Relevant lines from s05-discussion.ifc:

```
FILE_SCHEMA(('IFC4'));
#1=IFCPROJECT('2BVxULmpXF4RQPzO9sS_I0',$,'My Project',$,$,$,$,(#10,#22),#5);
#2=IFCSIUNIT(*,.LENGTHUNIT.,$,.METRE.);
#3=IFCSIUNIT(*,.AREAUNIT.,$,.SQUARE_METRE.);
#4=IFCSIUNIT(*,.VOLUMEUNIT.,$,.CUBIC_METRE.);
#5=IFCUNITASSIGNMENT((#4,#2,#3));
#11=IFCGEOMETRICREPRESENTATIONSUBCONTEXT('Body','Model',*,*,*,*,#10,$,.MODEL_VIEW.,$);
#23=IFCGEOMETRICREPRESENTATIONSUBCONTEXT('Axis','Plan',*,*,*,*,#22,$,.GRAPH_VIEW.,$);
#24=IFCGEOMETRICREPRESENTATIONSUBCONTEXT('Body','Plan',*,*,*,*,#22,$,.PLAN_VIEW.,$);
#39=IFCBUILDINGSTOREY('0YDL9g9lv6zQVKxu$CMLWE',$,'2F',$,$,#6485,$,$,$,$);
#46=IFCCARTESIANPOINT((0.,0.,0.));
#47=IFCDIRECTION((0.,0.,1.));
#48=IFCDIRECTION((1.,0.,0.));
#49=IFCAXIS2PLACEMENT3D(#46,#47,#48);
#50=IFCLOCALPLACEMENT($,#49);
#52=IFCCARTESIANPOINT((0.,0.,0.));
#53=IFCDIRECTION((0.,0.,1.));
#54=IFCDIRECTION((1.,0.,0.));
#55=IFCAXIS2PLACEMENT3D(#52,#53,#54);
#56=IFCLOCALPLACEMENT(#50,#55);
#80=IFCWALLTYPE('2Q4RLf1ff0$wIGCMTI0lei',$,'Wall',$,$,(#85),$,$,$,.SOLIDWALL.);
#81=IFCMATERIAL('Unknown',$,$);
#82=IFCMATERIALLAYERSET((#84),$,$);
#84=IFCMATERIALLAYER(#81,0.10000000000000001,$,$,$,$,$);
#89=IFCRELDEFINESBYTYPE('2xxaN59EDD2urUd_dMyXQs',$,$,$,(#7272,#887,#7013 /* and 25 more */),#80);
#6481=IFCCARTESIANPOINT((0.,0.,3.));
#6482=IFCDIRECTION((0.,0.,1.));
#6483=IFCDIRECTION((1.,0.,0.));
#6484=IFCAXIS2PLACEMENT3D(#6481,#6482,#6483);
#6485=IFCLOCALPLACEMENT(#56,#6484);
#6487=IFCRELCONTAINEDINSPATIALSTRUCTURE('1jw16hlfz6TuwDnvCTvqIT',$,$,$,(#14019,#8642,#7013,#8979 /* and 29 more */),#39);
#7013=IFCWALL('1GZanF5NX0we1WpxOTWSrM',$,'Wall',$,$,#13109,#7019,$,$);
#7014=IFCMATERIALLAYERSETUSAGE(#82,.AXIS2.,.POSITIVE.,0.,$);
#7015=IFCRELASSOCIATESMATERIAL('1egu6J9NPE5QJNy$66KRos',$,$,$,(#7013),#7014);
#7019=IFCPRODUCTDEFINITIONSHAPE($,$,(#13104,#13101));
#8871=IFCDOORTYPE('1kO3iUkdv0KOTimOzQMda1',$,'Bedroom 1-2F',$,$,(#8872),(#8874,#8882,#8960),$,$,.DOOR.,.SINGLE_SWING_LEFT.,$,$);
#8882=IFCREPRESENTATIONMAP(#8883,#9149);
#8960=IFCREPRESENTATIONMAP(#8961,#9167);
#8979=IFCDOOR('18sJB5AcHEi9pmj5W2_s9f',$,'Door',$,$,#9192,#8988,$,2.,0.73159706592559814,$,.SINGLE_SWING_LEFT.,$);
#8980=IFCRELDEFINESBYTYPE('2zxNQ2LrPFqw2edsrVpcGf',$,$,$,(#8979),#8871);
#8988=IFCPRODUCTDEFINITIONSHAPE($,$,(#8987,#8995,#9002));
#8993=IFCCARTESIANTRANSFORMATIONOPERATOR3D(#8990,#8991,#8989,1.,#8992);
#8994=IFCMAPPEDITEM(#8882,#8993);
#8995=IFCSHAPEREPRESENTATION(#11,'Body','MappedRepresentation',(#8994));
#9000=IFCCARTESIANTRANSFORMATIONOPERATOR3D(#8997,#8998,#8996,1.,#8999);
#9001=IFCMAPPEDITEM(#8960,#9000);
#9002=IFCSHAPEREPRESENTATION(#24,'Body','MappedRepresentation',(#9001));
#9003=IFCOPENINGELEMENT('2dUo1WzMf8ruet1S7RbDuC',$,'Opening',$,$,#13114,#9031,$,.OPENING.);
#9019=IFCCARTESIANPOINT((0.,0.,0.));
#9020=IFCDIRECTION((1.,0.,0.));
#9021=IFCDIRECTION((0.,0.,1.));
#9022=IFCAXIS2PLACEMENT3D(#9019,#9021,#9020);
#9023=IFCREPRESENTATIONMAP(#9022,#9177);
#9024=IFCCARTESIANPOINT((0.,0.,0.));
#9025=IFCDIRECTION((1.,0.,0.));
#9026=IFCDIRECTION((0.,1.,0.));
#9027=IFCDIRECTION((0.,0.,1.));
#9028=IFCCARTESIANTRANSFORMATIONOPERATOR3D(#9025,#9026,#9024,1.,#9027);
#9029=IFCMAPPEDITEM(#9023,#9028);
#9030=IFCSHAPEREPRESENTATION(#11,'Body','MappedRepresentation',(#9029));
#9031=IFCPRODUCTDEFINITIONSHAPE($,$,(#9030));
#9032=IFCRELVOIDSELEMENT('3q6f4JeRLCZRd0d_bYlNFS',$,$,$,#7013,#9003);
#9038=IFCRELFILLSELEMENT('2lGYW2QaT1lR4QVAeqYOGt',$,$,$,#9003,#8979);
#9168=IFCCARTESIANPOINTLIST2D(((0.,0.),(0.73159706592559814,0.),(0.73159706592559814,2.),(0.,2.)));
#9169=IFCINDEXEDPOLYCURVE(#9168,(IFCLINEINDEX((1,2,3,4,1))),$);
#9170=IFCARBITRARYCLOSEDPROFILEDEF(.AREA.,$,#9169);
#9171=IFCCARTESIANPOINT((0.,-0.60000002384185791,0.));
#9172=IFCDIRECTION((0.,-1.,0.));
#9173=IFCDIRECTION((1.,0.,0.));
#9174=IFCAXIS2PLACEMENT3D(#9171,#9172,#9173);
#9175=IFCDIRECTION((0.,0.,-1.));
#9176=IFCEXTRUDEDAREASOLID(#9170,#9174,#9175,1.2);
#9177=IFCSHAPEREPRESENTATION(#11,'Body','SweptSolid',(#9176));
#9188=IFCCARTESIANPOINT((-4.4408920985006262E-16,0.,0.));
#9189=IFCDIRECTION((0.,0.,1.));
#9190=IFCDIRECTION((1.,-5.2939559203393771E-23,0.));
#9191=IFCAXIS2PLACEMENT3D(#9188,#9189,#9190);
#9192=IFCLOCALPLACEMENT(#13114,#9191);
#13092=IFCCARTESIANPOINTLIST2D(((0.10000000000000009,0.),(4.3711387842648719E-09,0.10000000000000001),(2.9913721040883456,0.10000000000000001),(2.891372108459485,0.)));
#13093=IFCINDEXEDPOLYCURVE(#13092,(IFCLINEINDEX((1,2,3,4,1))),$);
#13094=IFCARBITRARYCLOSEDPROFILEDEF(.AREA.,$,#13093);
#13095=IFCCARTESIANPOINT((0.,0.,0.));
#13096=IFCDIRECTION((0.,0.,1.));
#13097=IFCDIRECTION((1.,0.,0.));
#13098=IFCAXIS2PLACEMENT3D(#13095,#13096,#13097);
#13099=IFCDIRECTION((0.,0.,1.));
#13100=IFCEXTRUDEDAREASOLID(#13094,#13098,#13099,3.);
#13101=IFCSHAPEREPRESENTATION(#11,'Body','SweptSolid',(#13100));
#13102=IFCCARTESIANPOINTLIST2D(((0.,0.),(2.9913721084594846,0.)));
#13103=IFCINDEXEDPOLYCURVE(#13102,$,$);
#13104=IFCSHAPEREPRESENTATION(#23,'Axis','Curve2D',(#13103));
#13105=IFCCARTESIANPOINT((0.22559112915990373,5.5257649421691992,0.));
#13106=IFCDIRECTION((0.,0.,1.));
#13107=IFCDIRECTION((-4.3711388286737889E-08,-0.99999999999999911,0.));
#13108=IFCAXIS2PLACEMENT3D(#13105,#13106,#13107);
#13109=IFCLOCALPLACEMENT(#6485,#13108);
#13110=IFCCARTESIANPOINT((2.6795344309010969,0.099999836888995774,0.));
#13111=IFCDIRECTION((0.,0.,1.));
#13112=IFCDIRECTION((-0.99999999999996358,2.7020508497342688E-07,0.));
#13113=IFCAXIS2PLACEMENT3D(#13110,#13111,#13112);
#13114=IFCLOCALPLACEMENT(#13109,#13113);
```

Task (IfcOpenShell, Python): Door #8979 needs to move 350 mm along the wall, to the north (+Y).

```python
import ifcopenshell
import ifcopenshell.api.geometry
import ifcopenshell.util.placement
import ifcopenshell.util.unit

model = ifcopenshell.open("s05-discussion.ifc")
unit_scale = ifcopenshell.util.unit.calculate_unit_scale(model)

door = model.by_guid("18sJB5AcHEi9pmj5W2_s9f")
opening = door.FillsVoids[0].RelatingOpeningElement
wall = opening.VoidsElements[0].RelatingBuildingElement

wall_matrix = ifcopenshell.util.placement.get_local_placement(wall.ObjectPlacement)
shift = wall_matrix[:3, 0] * -0.35 / unit_scale
before = ifcopenshell.util.placement.get_local_placement(door.ObjectPlacement)[:3, 3].copy()

# The door is placed relative to its opening, so it follows when the opening moves.
matrix = ifcopenshell.util.placement.get_local_placement(opening.ObjectPlacement)
matrix[:3, 3] += shift
ifcopenshell.api.geometry.edit_object_placement(
    model, product=opening, matrix=matrix, is_si=False, should_transform_children=True
)

after = ifcopenshell.util.placement.get_local_placement(door.ObjectPlacement)[:3, 3]
print("door moved by", (after - before).round(3) + 0.0)

model.write("s05-discussion_rev.ifc")
```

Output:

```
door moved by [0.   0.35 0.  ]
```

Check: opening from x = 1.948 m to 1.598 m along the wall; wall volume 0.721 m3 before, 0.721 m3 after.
